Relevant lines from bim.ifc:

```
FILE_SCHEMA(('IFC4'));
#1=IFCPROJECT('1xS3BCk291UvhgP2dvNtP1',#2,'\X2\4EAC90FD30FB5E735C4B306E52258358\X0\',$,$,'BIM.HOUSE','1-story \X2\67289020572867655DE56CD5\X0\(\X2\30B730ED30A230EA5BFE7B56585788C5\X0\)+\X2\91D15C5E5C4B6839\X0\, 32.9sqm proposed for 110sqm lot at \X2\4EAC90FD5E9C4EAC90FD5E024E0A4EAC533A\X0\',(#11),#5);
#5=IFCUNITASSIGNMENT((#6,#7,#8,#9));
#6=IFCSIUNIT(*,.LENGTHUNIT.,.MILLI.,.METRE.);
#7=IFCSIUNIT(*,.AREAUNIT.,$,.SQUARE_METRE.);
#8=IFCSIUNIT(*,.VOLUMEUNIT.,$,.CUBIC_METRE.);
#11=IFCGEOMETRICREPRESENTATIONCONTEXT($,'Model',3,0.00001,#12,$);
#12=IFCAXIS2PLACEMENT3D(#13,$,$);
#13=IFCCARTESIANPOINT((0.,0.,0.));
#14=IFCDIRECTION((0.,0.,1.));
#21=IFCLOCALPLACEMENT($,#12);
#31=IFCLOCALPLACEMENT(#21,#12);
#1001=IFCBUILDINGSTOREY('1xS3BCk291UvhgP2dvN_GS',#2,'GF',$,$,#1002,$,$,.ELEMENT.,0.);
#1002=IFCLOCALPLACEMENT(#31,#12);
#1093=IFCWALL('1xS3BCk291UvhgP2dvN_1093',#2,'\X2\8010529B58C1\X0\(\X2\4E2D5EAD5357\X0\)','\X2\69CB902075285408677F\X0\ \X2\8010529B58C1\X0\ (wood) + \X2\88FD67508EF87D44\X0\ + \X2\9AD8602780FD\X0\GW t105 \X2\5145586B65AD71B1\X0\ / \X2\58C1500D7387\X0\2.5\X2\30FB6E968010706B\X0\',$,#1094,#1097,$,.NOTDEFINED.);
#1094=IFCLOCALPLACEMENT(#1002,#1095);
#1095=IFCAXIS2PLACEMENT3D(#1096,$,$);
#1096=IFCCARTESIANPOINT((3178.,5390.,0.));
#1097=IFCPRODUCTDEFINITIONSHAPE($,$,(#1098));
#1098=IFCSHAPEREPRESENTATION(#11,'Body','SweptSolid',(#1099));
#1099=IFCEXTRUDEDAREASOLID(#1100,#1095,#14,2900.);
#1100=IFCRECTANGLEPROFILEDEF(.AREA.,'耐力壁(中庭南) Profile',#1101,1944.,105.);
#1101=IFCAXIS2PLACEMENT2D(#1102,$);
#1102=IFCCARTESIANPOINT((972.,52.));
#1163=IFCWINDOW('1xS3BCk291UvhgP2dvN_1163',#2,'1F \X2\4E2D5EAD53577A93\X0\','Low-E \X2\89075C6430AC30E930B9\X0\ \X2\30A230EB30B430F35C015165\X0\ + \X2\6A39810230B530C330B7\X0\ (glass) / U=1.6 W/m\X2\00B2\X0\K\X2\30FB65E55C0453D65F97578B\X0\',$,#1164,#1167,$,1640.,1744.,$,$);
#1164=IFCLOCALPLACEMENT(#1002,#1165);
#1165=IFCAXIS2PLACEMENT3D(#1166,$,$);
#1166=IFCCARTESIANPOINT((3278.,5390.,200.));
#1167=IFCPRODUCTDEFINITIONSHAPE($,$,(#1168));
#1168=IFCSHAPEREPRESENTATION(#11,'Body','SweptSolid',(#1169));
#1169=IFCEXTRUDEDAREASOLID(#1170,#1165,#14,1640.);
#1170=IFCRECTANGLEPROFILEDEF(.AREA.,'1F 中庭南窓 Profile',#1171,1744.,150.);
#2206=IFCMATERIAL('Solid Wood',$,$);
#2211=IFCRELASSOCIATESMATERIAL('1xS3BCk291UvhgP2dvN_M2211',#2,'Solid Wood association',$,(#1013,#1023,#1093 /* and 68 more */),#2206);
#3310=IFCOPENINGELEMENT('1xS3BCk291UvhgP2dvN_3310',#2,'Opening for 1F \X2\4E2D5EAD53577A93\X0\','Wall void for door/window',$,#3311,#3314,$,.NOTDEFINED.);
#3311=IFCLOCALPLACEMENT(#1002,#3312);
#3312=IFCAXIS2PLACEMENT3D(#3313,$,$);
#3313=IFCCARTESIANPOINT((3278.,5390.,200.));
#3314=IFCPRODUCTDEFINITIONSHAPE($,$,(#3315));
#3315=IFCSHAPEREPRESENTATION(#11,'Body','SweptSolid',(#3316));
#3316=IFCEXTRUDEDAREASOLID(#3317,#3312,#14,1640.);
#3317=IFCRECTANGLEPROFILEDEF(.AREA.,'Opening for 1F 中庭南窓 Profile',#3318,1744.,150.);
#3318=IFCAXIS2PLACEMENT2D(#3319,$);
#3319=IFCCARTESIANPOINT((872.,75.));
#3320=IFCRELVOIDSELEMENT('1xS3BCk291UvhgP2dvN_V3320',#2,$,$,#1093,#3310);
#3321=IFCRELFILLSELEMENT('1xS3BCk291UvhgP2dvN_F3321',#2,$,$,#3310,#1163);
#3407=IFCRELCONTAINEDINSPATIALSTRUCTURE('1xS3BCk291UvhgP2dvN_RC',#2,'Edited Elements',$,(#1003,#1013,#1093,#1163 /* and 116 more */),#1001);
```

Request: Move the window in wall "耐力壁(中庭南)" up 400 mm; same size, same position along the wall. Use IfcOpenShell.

```python
import numpy as np
import ifcopenshell
import ifcopenshell.api.geometry
import ifcopenshell.util.placement
import ifcopenshell.util.unit

model = ifcopenshell.open("bim.ifc")
unit_scale = ifcopenshell.util.unit.calculate_unit_scale(model)

window = model.by_guid("1xS3BCk291UvhgP2dvN_1163")
opening = window.FillsVoids[0].RelatingOpeningElement
dz = 0.4 / unit_scale

shift = np.array([0.0, 0.0, dz])
# The window is not placed relative to its opening, so move both.
for product in (opening, window):
    matrix = ifcopenshell.util.placement.get_local_placement(product.ObjectPlacement)
    matrix[:3, 3] += shift
    ifcopenshell.api.geometry.edit_object_placement(model, product=product, matrix=matrix, is_si=False)

print(f"moved by {dz * unit_scale:+.3f} m")

model.write("bim_edited.ifc")
```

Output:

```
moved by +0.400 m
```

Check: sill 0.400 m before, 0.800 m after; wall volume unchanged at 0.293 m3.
